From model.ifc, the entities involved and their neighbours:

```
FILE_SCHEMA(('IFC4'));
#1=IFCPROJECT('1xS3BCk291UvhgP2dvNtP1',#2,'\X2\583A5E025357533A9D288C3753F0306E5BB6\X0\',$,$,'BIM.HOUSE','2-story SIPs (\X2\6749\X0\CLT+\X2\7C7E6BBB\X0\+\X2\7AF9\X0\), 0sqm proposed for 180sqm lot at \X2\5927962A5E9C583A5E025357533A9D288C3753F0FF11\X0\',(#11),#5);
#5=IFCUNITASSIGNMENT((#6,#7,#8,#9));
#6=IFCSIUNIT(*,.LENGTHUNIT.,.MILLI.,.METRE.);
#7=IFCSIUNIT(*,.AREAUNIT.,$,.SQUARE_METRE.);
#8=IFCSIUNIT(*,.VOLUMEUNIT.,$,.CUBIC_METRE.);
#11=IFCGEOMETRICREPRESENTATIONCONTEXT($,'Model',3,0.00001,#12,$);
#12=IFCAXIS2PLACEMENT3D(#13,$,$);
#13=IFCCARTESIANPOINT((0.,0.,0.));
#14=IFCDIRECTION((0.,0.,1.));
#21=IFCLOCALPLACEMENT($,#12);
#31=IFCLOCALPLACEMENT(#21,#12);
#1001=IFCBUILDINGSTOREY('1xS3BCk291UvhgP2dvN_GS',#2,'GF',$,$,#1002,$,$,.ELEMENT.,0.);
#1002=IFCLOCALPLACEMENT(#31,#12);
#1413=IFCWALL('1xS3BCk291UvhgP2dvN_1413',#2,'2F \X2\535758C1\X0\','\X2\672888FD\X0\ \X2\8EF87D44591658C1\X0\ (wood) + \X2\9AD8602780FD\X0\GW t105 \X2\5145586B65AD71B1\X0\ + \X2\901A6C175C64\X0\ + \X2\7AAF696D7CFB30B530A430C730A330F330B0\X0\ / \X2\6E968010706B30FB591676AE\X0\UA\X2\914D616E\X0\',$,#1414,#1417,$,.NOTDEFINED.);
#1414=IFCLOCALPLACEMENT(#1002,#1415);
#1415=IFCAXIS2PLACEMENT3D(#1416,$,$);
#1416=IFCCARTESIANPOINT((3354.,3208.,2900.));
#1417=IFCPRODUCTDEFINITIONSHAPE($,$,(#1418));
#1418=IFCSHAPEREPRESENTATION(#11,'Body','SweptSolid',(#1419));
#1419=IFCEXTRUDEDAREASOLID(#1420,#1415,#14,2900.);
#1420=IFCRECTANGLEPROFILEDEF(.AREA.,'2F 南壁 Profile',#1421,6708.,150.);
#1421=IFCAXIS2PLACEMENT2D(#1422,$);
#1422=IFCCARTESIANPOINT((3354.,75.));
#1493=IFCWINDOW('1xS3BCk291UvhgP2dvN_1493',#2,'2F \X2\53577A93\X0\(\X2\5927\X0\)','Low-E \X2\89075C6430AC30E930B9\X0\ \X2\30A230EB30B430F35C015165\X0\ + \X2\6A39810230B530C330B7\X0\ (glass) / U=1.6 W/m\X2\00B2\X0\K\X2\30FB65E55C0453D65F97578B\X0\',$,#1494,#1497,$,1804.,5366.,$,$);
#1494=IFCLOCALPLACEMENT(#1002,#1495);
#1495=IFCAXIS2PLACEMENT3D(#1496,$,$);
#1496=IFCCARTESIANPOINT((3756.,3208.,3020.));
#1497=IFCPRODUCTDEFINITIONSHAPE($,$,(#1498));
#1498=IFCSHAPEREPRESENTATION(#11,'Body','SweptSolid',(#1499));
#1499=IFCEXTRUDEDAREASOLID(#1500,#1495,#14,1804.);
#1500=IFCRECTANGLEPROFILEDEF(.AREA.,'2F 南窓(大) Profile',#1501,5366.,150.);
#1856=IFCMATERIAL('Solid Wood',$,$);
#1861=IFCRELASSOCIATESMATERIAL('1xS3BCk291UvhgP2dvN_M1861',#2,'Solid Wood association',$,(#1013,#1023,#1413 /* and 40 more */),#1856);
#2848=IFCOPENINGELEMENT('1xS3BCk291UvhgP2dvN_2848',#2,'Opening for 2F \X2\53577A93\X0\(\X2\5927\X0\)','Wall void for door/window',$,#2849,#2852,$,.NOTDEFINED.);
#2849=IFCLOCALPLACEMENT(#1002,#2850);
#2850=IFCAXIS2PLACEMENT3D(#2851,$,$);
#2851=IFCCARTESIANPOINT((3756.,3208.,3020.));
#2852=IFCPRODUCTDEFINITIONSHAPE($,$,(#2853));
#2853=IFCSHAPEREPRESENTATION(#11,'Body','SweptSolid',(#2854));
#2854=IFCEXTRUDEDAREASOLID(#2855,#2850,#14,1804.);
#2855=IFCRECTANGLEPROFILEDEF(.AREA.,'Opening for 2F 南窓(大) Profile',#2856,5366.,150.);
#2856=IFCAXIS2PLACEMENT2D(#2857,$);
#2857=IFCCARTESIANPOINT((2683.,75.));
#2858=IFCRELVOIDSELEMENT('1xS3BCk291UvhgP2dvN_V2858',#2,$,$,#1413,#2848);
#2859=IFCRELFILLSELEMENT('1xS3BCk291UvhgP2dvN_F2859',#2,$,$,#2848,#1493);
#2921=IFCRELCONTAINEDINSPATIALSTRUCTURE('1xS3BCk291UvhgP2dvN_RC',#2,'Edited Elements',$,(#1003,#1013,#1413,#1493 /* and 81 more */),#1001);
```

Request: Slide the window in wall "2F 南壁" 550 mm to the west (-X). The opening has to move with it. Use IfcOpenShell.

```python
import ifcopenshell
import ifcopenshell.api.geometry
import ifcopenshell.util.placement
import ifcopenshell.util.unit

model = ifcopenshell.open("model.ifc")
unit_scale = ifcopenshell.util.unit.calculate_unit_scale(model)

window = model.by_id(1493)
opening = window.FillsVoids[0].RelatingOpeningElement
wall = opening.VoidsElements[0].RelatingBuildingElement

wall_matrix = ifcopenshell.util.placement.get_local_placement(wall.ObjectPlacement)
shift = wall_matrix[:3, 0] * -0.55 / unit_scale
before = ifcopenshell.util.placement.get_local_placement(window.ObjectPlacement)[:3, 3].copy()

# The window is not placed relative to its opening, so move both.
for product in (opening, window):
    matrix = ifcopenshell.util.placement.get_local_placement(product.ObjectPlacement)
    matrix[:3, 3] += shift
    ifcopenshell.api.geometry.edit_object_placement(model, product=product, matrix=matrix, is_si=False)

after = ifcopenshell.util.placement.get_local_placement(window.ObjectPlacement)[:3, 3]
print("window moved by", (after - before).round(3) + 0.0)

model.write("model_rev.ifc")
```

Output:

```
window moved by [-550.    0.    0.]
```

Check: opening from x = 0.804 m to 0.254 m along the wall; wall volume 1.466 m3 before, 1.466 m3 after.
